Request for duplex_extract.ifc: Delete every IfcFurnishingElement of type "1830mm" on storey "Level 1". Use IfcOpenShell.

First a look at what the model holds.

```python
import ifcopenshell
import ifcopenshell.util.element

model = ifcopenshell.open("duplex_extract.ifc")
print(model.schema)
storey = next(s for s in model.by_type("IfcBuildingStorey") if s.Name == "Level 1")
furniture = [e for e in ifcopenshell.util.element.get_decomposition(storey) if e.is_a("IfcFurnishingElement")]
seen = {}
for e in furniture:
    element_type = ifcopenshell.util.element.get_type(e)
    name = element_type.Name if element_type not in (None, e) else None
    seen[name] = seen.get(name, 0) + 1
for name, count in sorted(seen.items(), key=str):
    print(count, "x", name)
```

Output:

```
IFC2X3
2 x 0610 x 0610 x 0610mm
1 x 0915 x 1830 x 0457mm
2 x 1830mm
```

```python
import ifcopenshell
import ifcopenshell.api.root
import ifcopenshell.util.element

model = ifcopenshell.open("duplex_extract.ifc")

storey = next(s for s in model.by_type("IfcBuildingStorey") if s.Name == "Level 1")
furniture = [e for e in ifcopenshell.util.element.get_decomposition(storey) if e.is_a("IfcFurnishingElement")]
targets = [e for e in furniture if (t := ifcopenshell.util.element.get_type(e)) not in (None, e) and t.Name == "1830mm"]

for e in targets:
    ifcopenshell.api.root.remove_product(model, product=e)
print(len(targets), "removed")

model.write("duplex_extract_rev.ifc")
```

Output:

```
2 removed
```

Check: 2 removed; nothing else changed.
